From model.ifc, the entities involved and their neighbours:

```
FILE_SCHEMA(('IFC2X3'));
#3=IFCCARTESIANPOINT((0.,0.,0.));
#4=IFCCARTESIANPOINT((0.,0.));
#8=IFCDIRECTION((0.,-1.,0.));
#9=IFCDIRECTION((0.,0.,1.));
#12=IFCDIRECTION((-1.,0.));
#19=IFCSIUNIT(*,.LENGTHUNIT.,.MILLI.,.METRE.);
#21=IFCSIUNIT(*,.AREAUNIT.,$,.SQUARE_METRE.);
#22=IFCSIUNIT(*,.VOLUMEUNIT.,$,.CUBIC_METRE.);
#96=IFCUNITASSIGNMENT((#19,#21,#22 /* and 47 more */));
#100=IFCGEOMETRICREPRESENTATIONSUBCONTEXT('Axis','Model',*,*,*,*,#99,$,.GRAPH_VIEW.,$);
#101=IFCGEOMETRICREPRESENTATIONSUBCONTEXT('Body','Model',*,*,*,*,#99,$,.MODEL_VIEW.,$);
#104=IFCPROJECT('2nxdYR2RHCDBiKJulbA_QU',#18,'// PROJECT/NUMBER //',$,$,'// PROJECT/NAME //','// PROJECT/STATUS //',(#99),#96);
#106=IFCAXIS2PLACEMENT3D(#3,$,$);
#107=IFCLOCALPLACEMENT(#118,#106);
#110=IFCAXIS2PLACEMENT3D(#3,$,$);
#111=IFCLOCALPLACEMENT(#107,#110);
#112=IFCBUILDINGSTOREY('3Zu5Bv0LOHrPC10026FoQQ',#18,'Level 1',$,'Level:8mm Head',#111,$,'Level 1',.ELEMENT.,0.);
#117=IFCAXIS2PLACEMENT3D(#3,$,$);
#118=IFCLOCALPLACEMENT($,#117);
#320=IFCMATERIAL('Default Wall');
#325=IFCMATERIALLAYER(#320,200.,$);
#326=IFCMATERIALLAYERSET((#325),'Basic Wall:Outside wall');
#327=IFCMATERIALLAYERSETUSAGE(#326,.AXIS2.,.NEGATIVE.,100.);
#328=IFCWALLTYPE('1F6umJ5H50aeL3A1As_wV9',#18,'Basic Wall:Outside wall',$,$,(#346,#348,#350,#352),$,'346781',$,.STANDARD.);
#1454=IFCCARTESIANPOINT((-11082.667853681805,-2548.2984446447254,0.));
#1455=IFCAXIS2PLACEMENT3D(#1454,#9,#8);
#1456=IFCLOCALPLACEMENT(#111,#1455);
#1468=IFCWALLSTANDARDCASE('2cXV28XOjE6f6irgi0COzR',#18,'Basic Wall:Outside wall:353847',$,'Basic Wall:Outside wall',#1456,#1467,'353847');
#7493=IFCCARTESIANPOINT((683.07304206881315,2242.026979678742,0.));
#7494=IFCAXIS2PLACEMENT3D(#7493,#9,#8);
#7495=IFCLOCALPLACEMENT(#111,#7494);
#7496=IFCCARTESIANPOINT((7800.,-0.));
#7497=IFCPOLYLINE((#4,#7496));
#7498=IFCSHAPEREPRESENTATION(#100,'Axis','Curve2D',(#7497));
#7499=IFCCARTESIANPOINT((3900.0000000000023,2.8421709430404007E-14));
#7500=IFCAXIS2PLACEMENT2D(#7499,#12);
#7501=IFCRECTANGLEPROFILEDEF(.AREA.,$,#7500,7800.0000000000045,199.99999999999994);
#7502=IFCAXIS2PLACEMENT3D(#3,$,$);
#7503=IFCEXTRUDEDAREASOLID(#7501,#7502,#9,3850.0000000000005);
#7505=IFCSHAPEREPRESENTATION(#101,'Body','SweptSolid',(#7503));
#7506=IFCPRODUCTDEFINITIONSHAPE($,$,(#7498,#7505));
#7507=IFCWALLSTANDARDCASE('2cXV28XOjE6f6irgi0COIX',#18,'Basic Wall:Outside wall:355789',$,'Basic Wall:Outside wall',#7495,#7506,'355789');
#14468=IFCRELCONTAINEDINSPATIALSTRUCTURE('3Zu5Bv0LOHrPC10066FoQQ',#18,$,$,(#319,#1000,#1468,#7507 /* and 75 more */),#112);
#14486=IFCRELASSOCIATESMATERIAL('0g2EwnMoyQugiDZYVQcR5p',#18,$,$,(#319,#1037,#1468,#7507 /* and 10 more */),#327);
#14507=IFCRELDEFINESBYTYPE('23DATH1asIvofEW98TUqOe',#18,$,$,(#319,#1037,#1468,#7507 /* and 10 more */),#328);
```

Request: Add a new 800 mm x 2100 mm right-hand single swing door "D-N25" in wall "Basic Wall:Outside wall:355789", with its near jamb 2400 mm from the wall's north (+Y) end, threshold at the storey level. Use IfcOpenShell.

```python
import numpy as np
import ifcopenshell
import ifcopenshell.api.feature
import ifcopenshell.api.geometry
import ifcopenshell.api.root
import ifcopenshell.api.spatial
import ifcopenshell.api.type
import ifcopenshell.geom
import ifcopenshell.util.element
import ifcopenshell.util.placement
import ifcopenshell.util.representation
import ifcopenshell.util.shape
import ifcopenshell.util.unit

model = ifcopenshell.open("model.ifc")
unit_scale = ifcopenshell.util.unit.calculate_unit_scale(model)
settings = ifcopenshell.geom.settings()


def volume(element):
    """Net volume in cubic metres, openings subtracted."""
    shape = ifcopenshell.geom.create_shape(settings, element)
    return ifcopenshell.util.shape.get_volume(shape.geometry)


wall = model.by_id(7507)
storey = ifcopenshell.util.element.get_container(wall, ifc_class="IfcBuildingStorey")
context = ifcopenshell.util.representation.get_context(model, "Model", "Body", "MODEL_VIEW")
before = volume(wall)

width, height, from_end, sill = 0.8, 2.1, 2.4, 0.0  # metres

# The wall runs along its own X axis, and the end named is its -X end.
wall_shape = ifcopenshell.geom.create_shape(settings, wall)
x, y, z = ifcopenshell.util.shape.get_vertices(wall_shape.geometry).T
start = x.min() + from_end
face, thickness = float(y.min()), float(y.max() - y.min())
wall_matrix = ifcopenshell.util.placement.get_local_placement(wall.ObjectPlacement)
level = ifcopenshell.util.placement.get_local_placement(storey.ObjectPlacement)[2, 3]


def in_wall(x, y):
    """Placement at x, y metres in the wall's axes, at sill height."""
    matrix = wall_matrix.copy()
    matrix[:, 3] = wall_matrix @ np.array([x / unit_scale, y / unit_scale, 0.0, 1.0])
    matrix[2, 3] = level + sill / unit_scale
    return matrix


# Opening: a box that overshoots both wall faces by 50 mm.
opening = ifcopenshell.api.root.create_entity(model, ifc_class="IfcOpeningElement")
box = ifcopenshell.api.geometry.add_wall_representation(
    model, context=context, length=width, height=height, thickness=thickness + 0.1
)
ifcopenshell.api.geometry.assign_representation(model, product=opening, representation=box)
ifcopenshell.api.geometry.edit_object_placement(model, product=opening, matrix=in_wall(start, face - 0.05), is_si=False)
ifcopenshell.api.feature.add_feature(model, feature=opening, element=wall)

door = ifcopenshell.api.root.create_entity(model, ifc_class="IfcDoor", name="D-N25")
door.OverallWidth, door.OverallHeight = width / unit_scale, height / unit_scale
body = ifcopenshell.api.geometry.add_door_representation(
    model,
    context=context,
    overall_width=door.OverallWidth,
    overall_height=door.OverallHeight,
    operation_type="SINGLE_SWING_RIGHT",
    lining_properties={"LiningDepth": thickness / unit_scale, "ThresholdDepth": thickness / unit_scale},
)
ifcopenshell.api.geometry.assign_representation(model, product=door, representation=body)
ifcopenshell.api.spatial.assign_container(model, products=[door], relating_structure=storey)
fills = ifcopenshell.api.feature.add_filling(model, opening=opening, element=door)
fills.OwnerHistory = door.OwnerHistory  # required in IFC2X3

# IFC2X3 keeps the operation on the door style.
style = ifcopenshell.api.root.create_entity(model, ifc_class="IfcDoorStyle", name="D-N25")
style.OperationType, style.ConstructionType = "SINGLE_SWING_RIGHT", "NOTDEFINED"
style.ParameterTakesPrecedence = style.Sizeable = False
ifcopenshell.api.type.assign_type(model, related_objects=[door], relating_type=style)

# The lining spans the wall, so the door starts at the wall face.
ifcopenshell.api.geometry.edit_object_placement(model, product=door, matrix=in_wall(start, face), is_si=False)

after = volume(wall)

print(f"wall volume {before:.3f} -> {after:.3f} m3")

model.write("model_rev.ifc")
```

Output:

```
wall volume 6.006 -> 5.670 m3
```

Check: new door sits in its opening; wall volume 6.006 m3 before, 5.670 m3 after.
